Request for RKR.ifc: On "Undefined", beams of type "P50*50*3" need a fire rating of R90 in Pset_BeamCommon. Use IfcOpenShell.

First a look at what the model holds.

```python
import ifcopenshell
import ifcopenshell.util.element

model = ifcopenshell.open("RKR.ifc")
print(model.schema)
storey = next(s for s in model.by_type("IfcBuildingStorey") if s.Name == "Undefined")
beams = [e for e in ifcopenshell.util.element.get_decomposition(storey) if e.is_a("IfcBeam")]
seen = {}
for e in beams:
    element_type = ifcopenshell.util.element.get_type(e)
    key = (element_type.Name if element_type != e and element_type else None, ifcopenshell.util.element.get_pset(e, "Pset_BeamCommon", "FireRating"))
    seen[key] = seen.get(key, 0) + 1
for (name, value), count in sorted(seen.items(), key=str):
    print(count, "x", name, "|", value)
```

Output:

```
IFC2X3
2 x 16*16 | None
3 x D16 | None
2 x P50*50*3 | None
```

```python
import ifcopenshell
import ifcopenshell.api.pset
import ifcopenshell.util.element

model = ifcopenshell.open("RKR.ifc")

storey = next(s for s in model.by_type("IfcBuildingStorey") if s.Name == "Undefined")
beams = [e for e in ifcopenshell.util.element.get_decomposition(storey) if e.is_a("IfcBeam")]

count = 0
for e in beams:
    element_type = ifcopenshell.util.element.get_type(e)
    if element_type in (None, e) or element_type.Name != "P50*50*3":
        continue
    # add_pset returns the element's existing set when there is one.
    pset = ifcopenshell.api.pset.add_pset(model, product=e, name="Pset_BeamCommon")
    ifcopenshell.api.pset.edit_pset(model, pset=pset, properties={"FireRating": "R90"})
    count += 1

print(count, "beams updated")

model.write("RKR_updated.ifc")
```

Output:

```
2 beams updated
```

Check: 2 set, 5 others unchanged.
